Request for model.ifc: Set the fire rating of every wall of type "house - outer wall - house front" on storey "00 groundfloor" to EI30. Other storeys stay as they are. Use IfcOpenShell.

First a look at what the model holds.

```python
import ifcopenshell
import ifcopenshell.util.element

model = ifcopenshell.open("model.ifc")
print(model.schema)
storey = next(s for s in model.by_type("IfcBuildingStorey") if s.Name == "00 groundfloor")
walls = [e for e in ifcopenshell.util.element.get_decomposition(storey) if e.is_a("IfcWall")]
seen = {}
for e in walls:
    element_type = ifcopenshell.util.element.get_type(e)
    key = (element_type.Name if element_type != e and element_type else None, ifcopenshell.util.element.get_pset(e, "Pset_WallCommon", "FireRating"))
    seen[key] = seen.get(key, 0) + 1
for (name, value), count in sorted(seen.items(), key=str):
    print(count, "x", name, "|", value)
```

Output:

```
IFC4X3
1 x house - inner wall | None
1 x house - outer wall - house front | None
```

```python
import ifcopenshell
import ifcopenshell.api.pset
import ifcopenshell.util.element

model = ifcopenshell.open("model.ifc")

storey = next(s for s in model.by_type("IfcBuildingStorey") if s.Name == "00 groundfloor")
walls = [e for e in ifcopenshell.util.element.get_decomposition(storey) if e.is_a("IfcWall")]

count = 0
for e in walls:
    element_type = ifcopenshell.util.element.get_type(e)
    if element_type in (None, e) or element_type.Name != "house - outer wall - house front":
        continue
    # add_pset returns the element's existing set when there is one.
    pset = ifcopenshell.api.pset.add_pset(model, product=e, name="Pset_WallCommon")
    ifcopenshell.api.pset.edit_pset(model, pset=pset, properties={"FireRating": "EI30"})
    count += 1

print(count, "walls updated")

model.write("model_edited.ifc")
```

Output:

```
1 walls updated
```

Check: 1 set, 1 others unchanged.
